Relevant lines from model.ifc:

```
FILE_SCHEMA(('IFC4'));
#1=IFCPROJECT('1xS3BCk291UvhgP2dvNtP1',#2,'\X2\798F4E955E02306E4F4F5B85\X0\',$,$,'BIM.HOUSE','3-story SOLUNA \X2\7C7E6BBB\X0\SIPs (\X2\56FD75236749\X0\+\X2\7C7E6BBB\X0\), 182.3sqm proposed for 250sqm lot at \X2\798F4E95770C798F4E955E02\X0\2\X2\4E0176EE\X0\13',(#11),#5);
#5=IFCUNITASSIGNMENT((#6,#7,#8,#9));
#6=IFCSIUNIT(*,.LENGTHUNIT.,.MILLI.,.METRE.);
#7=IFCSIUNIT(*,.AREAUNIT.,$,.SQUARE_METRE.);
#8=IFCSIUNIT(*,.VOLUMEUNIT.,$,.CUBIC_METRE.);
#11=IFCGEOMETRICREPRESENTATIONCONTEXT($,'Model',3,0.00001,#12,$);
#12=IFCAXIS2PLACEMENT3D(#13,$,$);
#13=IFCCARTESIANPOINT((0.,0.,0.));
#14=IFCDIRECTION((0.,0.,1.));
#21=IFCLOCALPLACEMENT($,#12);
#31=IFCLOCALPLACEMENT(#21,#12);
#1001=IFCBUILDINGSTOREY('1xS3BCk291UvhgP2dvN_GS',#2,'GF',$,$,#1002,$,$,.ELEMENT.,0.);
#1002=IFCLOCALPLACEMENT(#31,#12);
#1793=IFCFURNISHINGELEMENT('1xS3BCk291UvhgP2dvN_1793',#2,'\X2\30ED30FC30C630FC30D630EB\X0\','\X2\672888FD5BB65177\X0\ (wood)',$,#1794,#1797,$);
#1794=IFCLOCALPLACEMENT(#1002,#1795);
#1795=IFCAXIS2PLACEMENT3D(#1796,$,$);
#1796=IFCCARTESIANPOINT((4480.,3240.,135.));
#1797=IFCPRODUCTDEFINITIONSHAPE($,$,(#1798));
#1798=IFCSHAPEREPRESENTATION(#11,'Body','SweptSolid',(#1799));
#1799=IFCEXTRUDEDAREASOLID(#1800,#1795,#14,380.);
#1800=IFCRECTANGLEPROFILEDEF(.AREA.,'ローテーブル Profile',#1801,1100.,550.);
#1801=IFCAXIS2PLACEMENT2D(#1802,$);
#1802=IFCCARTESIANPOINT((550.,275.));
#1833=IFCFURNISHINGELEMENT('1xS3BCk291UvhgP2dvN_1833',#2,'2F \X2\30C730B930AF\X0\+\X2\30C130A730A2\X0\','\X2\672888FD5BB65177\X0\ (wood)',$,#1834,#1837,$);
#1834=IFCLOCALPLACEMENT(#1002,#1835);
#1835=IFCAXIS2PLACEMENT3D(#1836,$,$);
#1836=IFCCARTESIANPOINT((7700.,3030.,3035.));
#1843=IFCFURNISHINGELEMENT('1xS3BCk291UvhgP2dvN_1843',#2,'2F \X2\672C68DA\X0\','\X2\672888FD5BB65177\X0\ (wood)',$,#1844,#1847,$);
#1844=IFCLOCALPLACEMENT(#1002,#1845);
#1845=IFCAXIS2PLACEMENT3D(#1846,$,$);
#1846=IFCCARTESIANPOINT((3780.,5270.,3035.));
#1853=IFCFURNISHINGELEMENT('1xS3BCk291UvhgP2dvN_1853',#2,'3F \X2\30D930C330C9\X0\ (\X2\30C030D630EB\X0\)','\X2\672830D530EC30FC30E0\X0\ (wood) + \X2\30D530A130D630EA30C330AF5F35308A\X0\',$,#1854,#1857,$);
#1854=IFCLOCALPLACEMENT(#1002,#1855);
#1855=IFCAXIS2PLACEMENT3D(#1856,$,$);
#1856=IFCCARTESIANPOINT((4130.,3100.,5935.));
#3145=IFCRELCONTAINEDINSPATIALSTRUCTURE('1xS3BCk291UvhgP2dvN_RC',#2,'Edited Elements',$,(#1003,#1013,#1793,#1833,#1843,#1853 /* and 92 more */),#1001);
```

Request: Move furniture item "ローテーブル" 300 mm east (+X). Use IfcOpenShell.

```python
import ifcopenshell
import ifcopenshell.api.geometry
import ifcopenshell.util.placement

model = ifcopenshell.open("model.ifc")

item = model.by_id(1793)
matrix = ifcopenshell.util.placement.get_local_placement(item.ObjectPlacement)
matrix[0, 3] += 300.0
ifcopenshell.api.geometry.edit_object_placement(model, product=item, matrix=matrix, is_si=False)

print(ifcopenshell.util.placement.get_local_placement(item.ObjectPlacement).round(3) + 0.0)

model.write("model_edited.ifc")
```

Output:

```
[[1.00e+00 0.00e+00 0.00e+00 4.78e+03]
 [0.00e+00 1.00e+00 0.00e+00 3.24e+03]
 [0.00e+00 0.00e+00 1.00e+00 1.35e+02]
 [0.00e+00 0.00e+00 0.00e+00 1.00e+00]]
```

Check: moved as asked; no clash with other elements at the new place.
